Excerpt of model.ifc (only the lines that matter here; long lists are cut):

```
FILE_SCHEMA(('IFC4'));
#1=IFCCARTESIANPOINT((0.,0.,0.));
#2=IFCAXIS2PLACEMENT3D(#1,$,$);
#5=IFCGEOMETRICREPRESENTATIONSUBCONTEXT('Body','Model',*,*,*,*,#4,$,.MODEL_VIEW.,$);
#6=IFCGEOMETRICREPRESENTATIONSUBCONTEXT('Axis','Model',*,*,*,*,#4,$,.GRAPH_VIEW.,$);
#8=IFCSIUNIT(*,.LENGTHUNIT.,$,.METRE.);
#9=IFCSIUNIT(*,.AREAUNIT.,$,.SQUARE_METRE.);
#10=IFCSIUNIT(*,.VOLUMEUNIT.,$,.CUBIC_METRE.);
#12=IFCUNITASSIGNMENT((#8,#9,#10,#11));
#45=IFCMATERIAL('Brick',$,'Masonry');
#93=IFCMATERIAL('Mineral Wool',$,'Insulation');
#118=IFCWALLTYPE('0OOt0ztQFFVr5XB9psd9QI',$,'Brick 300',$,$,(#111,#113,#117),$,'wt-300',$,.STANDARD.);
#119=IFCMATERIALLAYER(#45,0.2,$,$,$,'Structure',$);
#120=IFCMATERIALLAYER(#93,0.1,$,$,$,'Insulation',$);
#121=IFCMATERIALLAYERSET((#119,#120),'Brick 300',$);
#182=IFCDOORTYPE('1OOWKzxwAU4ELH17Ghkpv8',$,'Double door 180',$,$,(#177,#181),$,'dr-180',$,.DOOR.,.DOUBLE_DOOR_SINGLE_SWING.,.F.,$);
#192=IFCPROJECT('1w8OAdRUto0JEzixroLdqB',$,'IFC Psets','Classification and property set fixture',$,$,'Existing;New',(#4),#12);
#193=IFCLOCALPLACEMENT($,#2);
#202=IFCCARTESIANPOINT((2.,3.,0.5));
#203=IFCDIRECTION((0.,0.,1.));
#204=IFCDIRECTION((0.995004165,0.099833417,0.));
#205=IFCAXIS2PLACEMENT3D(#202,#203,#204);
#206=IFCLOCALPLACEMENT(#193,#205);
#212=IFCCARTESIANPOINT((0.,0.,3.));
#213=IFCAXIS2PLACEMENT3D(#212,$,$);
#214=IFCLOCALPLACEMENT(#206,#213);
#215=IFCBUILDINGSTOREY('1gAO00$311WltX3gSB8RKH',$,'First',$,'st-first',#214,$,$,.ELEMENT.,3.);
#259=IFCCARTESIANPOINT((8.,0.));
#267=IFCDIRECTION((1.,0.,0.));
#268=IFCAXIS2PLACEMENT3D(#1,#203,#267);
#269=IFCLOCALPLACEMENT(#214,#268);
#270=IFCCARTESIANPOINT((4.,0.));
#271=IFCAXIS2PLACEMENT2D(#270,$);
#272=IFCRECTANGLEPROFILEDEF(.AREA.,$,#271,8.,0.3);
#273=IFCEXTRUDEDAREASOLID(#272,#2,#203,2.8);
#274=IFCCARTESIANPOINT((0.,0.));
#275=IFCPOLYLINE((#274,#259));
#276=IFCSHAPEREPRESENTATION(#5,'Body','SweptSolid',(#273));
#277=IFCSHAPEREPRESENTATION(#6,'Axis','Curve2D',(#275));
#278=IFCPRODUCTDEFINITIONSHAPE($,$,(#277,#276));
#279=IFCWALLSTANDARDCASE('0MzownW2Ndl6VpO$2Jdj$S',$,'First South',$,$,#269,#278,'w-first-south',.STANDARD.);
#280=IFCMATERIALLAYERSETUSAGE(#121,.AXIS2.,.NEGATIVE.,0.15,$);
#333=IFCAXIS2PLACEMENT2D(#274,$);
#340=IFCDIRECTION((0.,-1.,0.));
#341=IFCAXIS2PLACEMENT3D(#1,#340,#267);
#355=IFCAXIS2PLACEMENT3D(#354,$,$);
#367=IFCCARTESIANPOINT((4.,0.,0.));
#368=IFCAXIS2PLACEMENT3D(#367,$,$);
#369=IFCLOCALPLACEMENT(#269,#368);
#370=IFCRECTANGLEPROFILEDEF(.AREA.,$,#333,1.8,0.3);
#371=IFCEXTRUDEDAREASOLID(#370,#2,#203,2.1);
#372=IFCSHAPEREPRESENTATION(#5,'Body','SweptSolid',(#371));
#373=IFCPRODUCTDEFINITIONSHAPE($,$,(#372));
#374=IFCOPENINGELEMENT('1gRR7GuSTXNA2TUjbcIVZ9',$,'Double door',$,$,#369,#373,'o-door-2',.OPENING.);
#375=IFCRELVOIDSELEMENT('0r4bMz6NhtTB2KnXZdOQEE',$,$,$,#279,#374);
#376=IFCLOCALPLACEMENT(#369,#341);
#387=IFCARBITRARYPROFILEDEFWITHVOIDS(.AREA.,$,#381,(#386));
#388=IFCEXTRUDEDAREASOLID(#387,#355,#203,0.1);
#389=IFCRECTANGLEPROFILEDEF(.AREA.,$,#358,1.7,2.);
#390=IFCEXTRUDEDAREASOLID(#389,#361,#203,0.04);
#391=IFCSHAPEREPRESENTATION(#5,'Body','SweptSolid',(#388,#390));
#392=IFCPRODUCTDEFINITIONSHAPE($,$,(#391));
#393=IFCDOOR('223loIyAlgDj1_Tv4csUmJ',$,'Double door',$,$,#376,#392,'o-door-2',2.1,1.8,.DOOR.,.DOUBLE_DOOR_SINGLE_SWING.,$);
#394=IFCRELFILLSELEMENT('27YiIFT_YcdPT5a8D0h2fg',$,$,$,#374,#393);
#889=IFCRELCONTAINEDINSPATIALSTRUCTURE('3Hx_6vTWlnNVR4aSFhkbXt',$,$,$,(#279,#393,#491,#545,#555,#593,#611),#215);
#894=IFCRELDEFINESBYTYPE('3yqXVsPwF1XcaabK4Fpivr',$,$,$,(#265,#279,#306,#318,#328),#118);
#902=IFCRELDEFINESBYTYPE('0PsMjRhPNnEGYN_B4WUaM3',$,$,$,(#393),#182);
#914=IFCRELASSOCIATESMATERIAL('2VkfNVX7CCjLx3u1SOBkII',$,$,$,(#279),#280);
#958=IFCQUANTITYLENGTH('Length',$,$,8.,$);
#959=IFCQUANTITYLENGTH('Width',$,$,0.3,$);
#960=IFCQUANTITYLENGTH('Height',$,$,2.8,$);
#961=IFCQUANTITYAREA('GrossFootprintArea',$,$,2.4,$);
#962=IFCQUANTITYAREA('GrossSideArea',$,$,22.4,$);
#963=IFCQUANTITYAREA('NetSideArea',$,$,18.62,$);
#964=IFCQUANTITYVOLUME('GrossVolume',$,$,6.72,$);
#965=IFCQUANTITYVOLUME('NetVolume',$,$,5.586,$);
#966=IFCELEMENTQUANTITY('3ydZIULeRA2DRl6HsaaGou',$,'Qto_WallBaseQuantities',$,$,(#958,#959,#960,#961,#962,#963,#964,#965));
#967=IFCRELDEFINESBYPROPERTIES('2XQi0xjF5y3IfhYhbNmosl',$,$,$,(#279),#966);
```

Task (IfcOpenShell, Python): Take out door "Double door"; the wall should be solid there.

```python
import ifcopenshell
import ifcopenshell.api.feature
import ifcopenshell.api.pset
import ifcopenshell.api.root
import ifcopenshell.geom
import ifcopenshell.util.element
import ifcopenshell.util.shape
import ifcopenshell.util.unit

model = ifcopenshell.open("model.ifc")
area_scale = ifcopenshell.util.unit.calculate_unit_scale(model, "AREAUNIT")
volume_scale = ifcopenshell.util.unit.calculate_unit_scale(model, "VOLUMEUNIT")
settings = ifcopenshell.geom.settings()


def volume(element):
    """Net volume in cubic metres, openings subtracted."""
    shape = ifcopenshell.geom.create_shape(settings, element)
    return ifcopenshell.util.shape.get_volume(shape.geometry)


door = model.by_id(393)
opening = door.FillsVoids[0].RelatingOpeningElement
wall = opening.VoidsElements[0].RelatingBuildingElement
before = volume(wall)

ifcopenshell.api.root.remove_product(model, product=door)
ifcopenshell.api.feature.remove_feature(model, feature=opening)

after = volume(wall)
thickness = 0.3  # wall thickness in metres

# Update the wall's stored quantities.
qto = model.by_id(ifcopenshell.util.element.get_pset(wall, "Qto_WallBaseQuantities", should_inherit=False)["id"])
ifcopenshell.api.pset.edit_qto(model, qto=qto, properties={
    "NetSideArea": after / thickness / area_scale,
    "NetVolume": after / volume_scale,
})

print(f"wall volume {before:.3f} -> {after:.3f} m3")

model.write("model-out.ifc")
```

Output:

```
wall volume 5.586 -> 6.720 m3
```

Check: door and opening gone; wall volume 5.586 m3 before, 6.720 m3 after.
